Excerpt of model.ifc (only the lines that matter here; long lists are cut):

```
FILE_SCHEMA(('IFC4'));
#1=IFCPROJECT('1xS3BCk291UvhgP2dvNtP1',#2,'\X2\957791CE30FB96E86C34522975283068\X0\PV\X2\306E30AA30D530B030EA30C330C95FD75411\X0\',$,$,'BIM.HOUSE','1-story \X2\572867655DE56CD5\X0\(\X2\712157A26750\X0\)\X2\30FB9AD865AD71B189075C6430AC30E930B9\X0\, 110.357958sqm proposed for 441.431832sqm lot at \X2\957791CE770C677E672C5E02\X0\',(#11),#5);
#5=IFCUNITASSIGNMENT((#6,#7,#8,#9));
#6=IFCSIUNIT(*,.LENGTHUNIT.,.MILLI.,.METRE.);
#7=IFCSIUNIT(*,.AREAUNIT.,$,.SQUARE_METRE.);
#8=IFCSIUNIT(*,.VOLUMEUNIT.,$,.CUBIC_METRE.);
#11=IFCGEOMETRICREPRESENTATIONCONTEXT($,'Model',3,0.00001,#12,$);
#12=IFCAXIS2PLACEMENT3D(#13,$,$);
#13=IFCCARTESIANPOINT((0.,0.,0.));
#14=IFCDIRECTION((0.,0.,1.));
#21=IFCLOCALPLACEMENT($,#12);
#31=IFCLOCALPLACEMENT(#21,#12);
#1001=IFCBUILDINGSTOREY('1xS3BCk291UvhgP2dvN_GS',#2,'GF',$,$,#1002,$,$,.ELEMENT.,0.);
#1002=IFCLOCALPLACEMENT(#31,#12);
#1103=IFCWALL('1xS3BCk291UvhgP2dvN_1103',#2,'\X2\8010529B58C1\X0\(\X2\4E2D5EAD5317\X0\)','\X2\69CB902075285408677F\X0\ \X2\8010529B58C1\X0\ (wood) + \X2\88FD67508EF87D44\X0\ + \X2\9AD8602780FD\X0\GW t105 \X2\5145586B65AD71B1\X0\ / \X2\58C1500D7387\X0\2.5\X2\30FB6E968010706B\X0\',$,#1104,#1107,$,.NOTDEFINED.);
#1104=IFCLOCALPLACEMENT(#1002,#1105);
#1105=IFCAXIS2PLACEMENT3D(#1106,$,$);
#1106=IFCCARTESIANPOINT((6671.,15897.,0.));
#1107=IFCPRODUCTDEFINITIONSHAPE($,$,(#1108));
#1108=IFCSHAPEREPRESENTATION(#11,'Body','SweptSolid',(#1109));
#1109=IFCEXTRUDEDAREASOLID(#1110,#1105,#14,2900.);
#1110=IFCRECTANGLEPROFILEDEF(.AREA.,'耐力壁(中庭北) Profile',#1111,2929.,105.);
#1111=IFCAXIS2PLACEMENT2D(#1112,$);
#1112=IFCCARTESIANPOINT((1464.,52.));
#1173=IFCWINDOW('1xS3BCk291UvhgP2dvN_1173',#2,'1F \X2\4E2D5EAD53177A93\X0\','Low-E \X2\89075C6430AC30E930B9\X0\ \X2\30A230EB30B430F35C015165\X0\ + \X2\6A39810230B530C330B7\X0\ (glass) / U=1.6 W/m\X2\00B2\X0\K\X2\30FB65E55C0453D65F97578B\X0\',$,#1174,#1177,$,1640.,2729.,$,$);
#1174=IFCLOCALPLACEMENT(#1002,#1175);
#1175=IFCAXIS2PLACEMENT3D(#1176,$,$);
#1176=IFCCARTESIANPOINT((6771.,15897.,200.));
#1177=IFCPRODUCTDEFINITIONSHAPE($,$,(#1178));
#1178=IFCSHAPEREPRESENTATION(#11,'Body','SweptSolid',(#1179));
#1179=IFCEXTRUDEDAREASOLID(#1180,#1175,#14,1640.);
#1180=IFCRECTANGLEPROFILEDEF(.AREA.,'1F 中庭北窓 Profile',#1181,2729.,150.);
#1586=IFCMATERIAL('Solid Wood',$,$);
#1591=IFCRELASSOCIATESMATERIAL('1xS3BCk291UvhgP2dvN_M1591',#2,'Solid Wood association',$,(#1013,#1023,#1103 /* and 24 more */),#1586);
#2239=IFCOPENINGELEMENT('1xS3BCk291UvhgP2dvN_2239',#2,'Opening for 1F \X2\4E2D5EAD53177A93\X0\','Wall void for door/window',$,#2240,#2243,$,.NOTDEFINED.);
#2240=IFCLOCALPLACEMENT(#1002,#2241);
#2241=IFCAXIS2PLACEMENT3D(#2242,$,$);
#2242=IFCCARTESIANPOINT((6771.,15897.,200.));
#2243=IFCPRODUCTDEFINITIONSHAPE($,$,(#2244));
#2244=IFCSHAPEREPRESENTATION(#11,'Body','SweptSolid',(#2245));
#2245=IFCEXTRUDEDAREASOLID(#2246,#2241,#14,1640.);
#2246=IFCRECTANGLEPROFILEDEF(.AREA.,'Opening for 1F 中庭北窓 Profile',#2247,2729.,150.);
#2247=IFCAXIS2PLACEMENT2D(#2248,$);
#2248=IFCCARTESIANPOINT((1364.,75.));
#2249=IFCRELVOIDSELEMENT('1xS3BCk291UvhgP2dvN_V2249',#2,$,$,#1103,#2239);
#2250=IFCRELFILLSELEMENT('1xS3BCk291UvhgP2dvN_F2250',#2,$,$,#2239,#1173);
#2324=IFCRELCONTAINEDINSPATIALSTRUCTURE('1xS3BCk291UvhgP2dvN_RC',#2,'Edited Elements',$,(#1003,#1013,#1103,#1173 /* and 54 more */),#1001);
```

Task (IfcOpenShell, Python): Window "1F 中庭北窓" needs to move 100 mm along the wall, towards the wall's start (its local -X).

```python
import ifcopenshell
import ifcopenshell.api.geometry
import ifcopenshell.util.placement
import ifcopenshell.util.unit

model = ifcopenshell.open("model.ifc")
unit_scale = ifcopenshell.util.unit.calculate_unit_scale(model)

window = model.by_guid("1xS3BCk291UvhgP2dvN_1173")
opening = window.FillsVoids[0].RelatingOpeningElement
wall = opening.VoidsElements[0].RelatingBuildingElement

wall_matrix = ifcopenshell.util.placement.get_local_placement(wall.ObjectPlacement)
shift = wall_matrix[:3, 0] * -0.1 / unit_scale
before = ifcopenshell.util.placement.get_local_placement(window.ObjectPlacement)[:3, 3].copy()

# The window is not placed relative to its opening, so move both.
for product in (opening, window):
    matrix = ifcopenshell.util.placement.get_local_placement(product.ObjectPlacement)
    matrix[:3, 3] += shift
    ifcopenshell.api.geometry.edit_object_placement(model, product=product, matrix=matrix, is_si=False)

after = ifcopenshell.util.placement.get_local_placement(window.ObjectPlacement)[:3, 3]
print("window moved by", (after - before).round(3) + 0.0)

model.write("model_v2.ifc")
```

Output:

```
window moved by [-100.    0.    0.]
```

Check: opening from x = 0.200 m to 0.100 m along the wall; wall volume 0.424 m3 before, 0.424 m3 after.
